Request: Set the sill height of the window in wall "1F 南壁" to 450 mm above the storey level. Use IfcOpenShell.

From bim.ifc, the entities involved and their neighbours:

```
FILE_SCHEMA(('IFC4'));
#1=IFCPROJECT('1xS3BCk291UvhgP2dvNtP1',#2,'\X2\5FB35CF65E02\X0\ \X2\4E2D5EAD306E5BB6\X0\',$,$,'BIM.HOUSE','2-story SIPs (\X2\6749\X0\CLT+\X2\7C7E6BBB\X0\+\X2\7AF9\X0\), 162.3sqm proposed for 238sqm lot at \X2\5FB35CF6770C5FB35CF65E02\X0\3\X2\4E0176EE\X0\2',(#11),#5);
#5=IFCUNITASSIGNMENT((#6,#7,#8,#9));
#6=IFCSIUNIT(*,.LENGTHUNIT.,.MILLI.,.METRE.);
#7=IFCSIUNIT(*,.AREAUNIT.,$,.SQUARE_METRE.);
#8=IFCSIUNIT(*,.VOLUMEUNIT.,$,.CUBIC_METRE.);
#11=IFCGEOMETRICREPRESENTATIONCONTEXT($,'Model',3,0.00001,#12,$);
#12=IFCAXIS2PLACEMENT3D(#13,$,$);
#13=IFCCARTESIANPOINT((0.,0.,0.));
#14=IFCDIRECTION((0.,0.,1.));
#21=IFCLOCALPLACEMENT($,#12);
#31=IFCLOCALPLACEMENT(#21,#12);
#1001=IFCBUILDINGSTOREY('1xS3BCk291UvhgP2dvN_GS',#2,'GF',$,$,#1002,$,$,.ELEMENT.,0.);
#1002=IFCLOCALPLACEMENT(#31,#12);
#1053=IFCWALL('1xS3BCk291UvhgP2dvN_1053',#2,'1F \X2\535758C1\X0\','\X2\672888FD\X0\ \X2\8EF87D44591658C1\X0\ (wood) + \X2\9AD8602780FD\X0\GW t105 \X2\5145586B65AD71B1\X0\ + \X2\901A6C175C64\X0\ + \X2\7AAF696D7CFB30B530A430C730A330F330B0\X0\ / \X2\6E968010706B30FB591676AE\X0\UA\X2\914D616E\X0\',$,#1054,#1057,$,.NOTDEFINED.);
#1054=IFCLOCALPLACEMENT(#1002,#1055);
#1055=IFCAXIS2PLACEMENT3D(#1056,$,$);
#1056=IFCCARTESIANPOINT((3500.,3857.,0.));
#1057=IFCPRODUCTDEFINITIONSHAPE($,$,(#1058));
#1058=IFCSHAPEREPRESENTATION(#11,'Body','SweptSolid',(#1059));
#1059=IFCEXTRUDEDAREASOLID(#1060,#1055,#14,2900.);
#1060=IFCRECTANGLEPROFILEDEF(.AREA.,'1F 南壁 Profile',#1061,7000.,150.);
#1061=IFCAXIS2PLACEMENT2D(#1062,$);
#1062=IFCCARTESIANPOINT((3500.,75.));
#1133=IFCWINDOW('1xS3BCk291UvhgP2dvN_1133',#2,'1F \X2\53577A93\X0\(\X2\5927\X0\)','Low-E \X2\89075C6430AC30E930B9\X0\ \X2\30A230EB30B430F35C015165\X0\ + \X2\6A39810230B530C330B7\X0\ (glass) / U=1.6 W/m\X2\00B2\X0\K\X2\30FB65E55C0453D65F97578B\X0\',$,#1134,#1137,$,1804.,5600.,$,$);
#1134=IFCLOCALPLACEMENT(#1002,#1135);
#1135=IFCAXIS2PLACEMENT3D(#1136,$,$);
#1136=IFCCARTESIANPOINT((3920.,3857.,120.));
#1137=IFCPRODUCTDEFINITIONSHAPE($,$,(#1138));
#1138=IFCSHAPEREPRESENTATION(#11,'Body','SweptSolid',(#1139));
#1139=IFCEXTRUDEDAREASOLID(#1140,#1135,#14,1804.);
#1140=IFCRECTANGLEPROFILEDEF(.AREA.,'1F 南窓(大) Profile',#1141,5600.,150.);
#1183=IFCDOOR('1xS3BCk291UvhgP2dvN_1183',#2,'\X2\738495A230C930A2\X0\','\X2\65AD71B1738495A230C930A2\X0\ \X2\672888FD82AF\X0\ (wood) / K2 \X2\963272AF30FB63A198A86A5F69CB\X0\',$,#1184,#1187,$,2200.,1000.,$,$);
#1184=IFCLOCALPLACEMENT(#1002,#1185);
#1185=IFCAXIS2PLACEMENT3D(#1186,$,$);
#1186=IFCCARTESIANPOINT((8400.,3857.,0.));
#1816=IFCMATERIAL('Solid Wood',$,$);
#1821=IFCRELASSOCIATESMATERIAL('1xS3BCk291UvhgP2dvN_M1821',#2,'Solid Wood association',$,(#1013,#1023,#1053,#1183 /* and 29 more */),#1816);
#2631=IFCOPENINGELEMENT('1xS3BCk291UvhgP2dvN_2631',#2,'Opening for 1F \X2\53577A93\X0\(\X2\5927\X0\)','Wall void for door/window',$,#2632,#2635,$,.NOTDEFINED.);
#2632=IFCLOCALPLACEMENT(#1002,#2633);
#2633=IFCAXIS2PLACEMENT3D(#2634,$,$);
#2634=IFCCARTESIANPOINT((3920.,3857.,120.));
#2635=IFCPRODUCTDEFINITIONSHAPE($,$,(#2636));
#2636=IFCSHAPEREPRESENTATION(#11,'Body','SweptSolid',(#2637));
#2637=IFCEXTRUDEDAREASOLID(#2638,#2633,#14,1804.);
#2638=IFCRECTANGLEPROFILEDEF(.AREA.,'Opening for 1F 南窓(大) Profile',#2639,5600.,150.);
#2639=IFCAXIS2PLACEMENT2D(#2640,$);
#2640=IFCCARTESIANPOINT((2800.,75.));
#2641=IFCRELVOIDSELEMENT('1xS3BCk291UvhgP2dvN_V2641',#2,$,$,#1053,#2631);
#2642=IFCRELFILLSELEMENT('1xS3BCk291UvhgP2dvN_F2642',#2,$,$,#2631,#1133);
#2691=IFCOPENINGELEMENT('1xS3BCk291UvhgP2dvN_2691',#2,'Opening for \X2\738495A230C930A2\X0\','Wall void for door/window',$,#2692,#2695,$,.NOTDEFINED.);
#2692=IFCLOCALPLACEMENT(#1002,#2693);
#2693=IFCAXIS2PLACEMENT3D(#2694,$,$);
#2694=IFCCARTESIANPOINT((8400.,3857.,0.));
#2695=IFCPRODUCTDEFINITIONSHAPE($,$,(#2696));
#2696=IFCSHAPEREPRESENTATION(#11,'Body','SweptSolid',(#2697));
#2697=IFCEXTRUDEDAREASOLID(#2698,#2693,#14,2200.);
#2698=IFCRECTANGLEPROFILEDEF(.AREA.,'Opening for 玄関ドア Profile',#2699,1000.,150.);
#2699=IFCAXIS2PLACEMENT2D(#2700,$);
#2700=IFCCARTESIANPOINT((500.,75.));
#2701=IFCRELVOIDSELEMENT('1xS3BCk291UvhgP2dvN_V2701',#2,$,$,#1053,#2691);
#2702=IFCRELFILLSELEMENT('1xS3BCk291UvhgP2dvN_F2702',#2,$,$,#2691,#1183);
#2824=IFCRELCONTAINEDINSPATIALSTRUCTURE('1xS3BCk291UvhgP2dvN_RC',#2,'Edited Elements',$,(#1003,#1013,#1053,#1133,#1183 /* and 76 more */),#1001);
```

```python
import numpy as np
import ifcopenshell
import ifcopenshell.api.geometry
import ifcopenshell.geom
import ifcopenshell.util.element
import ifcopenshell.util.placement
import ifcopenshell.util.shape
import ifcopenshell.util.unit

model = ifcopenshell.open("bim.ifc")
unit_scale = ifcopenshell.util.unit.calculate_unit_scale(model)

window = model.by_guid("1xS3BCk291UvhgP2dvN_1133")
opening = window.FillsVoids[0].RelatingOpeningElement
storey = ifcopenshell.util.element.get_container(window, ifc_class="IfcBuildingStorey")
level = ifcopenshell.util.placement.get_local_placement(storey.ObjectPlacement)[2, 3]

# The opening's origin need not be at the sill, so measure its lowest point.
shape = ifcopenshell.geom.create_shape(ifcopenshell.geom.settings(), opening)
bottom = ifcopenshell.util.shape.get_shape_bottom_elevation(shape, shape.geometry) / unit_scale
dz = level + 0.45 / unit_scale - bottom

shift = np.array([0.0, 0.0, dz])
# The window is not placed relative to its opening, so move both.
for product in (opening, window):
    matrix = ifcopenshell.util.placement.get_local_placement(product.ObjectPlacement)
    matrix[:3, 3] += shift
    ifcopenshell.api.geometry.edit_object_placement(model, product=product, matrix=matrix, is_si=False)

print(f"moved by {dz * unit_scale:+.3f} m")

model.write("bim_rev.ifc")
```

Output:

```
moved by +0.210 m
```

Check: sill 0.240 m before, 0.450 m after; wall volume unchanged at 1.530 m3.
